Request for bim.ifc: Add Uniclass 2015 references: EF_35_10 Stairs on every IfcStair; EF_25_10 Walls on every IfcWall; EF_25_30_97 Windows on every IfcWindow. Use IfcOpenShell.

First a look at what the model holds.

```python
import ifcopenshell

model = ifcopenshell.open("bim.ifc")
print(model.schema)
print("classifications:", [c.Name for c in model.by_type("IfcClassification")])
for ifc_class in ("IfcDoor", "IfcRoof", "IfcStair", "IfcWall", "IfcWindow"):
    print(ifc_class, len(model.by_type(ifc_class)))
```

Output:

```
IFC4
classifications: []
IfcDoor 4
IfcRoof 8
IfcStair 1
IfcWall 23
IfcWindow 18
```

```python
import ifcopenshell
import ifcopenshell.api.classification

model = ifcopenshell.open("bim.ifc")

system = ifcopenshell.api.classification.add_classification(model, classification="Uniclass 2015")

codes = {
    "IfcStair": ("EF_35_10", "Stairs"),
    "IfcWall": ("EF_25_10", "Walls"),
    "IfcWindow": ("EF_25_30_97", "Windows"),
}
for ifc_class, (code, name) in codes.items():
    products = model.by_type(ifc_class)
    ifcopenshell.api.classification.add_reference(
        model, products=products, classification=system, identification=code, name=name
    )
    print(code, len(products))

model.write("bim_updated.ifc")
```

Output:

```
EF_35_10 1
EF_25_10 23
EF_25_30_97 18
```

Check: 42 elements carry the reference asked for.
